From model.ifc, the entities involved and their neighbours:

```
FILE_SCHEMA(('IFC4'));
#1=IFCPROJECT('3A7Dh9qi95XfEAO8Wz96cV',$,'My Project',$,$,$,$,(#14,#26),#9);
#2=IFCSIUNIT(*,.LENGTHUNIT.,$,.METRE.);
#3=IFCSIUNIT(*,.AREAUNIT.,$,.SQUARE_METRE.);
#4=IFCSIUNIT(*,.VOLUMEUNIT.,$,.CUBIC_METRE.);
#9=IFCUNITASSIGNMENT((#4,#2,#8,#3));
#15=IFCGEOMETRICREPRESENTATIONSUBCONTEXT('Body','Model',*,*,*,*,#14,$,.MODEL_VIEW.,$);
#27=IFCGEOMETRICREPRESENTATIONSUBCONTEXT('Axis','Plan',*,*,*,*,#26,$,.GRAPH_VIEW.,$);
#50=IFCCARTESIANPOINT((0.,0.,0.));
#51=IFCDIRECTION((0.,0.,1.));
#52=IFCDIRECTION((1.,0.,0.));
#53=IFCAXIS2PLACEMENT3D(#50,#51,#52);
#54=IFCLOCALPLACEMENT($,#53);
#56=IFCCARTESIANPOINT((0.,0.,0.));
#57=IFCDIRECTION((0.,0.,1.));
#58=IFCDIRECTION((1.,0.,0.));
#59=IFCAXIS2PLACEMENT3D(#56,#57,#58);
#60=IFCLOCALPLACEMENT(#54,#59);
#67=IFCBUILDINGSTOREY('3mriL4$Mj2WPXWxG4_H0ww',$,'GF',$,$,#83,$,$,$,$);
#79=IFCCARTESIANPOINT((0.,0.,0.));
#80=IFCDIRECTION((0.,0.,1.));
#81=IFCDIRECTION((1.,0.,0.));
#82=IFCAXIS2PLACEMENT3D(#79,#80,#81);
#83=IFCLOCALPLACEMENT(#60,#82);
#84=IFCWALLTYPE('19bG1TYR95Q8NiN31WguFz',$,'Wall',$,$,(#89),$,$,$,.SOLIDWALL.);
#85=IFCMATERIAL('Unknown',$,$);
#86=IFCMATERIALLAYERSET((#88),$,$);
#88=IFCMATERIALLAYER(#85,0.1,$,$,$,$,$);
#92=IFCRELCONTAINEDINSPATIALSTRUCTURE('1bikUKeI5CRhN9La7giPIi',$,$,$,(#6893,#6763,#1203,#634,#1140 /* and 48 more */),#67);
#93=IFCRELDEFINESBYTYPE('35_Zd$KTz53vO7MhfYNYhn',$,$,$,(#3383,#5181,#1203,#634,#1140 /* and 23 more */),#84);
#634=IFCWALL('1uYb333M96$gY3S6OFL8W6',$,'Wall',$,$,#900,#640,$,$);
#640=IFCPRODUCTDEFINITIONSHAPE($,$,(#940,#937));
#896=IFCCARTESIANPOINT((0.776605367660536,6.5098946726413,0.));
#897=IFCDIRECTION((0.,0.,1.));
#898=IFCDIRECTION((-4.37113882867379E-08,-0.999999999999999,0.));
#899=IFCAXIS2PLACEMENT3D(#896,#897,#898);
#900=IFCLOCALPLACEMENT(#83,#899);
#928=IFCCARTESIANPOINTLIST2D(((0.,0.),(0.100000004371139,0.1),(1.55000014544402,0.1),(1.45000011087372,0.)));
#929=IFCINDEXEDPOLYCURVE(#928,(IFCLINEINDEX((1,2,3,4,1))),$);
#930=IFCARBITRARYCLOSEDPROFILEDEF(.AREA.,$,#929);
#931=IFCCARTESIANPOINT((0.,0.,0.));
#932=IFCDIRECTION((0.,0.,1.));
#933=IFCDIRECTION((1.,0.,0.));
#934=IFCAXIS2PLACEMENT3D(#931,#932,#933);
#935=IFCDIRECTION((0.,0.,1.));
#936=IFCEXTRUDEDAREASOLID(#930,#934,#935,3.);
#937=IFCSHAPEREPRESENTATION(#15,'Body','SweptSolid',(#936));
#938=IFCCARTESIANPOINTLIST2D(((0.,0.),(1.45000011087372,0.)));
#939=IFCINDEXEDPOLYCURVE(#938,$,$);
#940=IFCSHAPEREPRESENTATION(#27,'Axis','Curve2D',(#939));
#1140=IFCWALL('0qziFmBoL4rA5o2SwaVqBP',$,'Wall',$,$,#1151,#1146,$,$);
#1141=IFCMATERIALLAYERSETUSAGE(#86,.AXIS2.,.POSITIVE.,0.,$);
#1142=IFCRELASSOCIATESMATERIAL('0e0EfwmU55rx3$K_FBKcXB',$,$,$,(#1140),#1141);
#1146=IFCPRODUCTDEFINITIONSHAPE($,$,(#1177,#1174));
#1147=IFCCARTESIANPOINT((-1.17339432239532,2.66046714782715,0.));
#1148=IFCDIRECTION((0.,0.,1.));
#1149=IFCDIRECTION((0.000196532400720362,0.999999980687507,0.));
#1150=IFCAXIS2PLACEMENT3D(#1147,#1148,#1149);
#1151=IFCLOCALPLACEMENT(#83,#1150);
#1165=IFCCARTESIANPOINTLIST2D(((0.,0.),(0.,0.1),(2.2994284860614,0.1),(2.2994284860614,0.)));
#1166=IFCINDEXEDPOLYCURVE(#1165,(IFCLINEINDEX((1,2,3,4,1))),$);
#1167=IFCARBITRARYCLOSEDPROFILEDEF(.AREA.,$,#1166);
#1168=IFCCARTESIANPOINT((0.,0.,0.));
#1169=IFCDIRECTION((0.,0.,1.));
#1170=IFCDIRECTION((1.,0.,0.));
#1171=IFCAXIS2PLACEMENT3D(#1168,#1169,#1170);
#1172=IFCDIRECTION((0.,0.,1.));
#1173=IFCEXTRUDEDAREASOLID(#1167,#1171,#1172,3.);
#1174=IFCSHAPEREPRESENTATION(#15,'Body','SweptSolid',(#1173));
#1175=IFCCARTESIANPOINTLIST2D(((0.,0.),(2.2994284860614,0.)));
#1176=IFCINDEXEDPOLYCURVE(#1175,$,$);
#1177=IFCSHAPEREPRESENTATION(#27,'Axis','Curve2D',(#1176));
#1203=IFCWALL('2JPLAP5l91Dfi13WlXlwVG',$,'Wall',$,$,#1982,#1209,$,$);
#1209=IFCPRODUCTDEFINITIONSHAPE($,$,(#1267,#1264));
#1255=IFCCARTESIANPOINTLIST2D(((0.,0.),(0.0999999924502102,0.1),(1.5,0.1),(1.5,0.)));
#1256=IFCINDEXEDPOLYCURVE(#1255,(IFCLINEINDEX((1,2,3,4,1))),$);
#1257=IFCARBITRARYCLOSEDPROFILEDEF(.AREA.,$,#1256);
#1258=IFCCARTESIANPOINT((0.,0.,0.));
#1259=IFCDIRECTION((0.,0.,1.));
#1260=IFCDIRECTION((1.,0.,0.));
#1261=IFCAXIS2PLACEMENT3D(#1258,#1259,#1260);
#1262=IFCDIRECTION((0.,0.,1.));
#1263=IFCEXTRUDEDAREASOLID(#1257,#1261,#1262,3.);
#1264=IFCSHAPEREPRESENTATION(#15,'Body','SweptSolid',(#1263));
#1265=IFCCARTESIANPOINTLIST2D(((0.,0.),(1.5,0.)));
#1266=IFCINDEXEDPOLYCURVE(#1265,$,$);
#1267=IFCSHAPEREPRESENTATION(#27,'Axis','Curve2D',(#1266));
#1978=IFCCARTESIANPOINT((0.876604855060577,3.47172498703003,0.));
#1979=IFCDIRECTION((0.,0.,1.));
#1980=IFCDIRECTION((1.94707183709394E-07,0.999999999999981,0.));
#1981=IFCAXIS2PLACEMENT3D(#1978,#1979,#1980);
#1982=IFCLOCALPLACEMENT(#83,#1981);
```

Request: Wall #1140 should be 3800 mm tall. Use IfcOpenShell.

```python
import ifcopenshell
import ifcopenshell.geom
import ifcopenshell.util.representation
import ifcopenshell.util.shape
import ifcopenshell.util.unit

model = ifcopenshell.open("model.ifc")
unit_scale = ifcopenshell.util.unit.calculate_unit_scale(model)
settings = ifcopenshell.geom.settings()


def volume(element):
    """Net volume in cubic metres, openings subtracted."""
    shape = ifcopenshell.geom.create_shape(settings, element)
    return ifcopenshell.util.shape.get_volume(shape.geometry)


wall = model.by_guid("0qziFmBoL4rA5o2SwaVqBP")
before = volume(wall)

body = ifcopenshell.util.representation.get_representation(wall, "Model", "Body")
solid = body.Items[0]
old_height = solid.Depth
solid.Depth = 3.8 / unit_scale
after = volume(wall)

print(f"height {old_height:g} -> {solid.Depth:g}, volume {before:.3f} -> {after:.3f} m3")

model.write("model-out.ifc")
```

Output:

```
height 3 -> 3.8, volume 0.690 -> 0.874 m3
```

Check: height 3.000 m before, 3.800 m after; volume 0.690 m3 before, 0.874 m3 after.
